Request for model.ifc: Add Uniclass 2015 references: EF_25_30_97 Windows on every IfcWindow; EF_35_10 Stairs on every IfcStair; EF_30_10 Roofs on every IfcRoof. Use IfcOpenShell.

First a look at what the model holds.

```python
import ifcopenshell

model = ifcopenshell.open("model.ifc")
print(model.schema)
print("classifications:", [c.Name for c in model.by_type("IfcClassification")])
for ifc_class in ("IfcDoor", "IfcRoof", "IfcStair", "IfcWall", "IfcWindow"):
    print(ifc_class, len(model.by_type(ifc_class)))
```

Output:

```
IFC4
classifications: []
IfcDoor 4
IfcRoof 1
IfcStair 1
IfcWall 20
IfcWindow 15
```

```python
import ifcopenshell
import ifcopenshell.api.classification

model = ifcopenshell.open("model.ifc")

system = ifcopenshell.api.classification.add_classification(model, classification="Uniclass 2015")

codes = {
    "IfcWindow": ("EF_25_30_97", "Windows"),
    "IfcStair": ("EF_35_10", "Stairs"),
    "IfcRoof": ("EF_30_10", "Roofs"),
}
for ifc_class, (code, name) in codes.items():
    products = model.by_type(ifc_class)
    ifcopenshell.api.classification.add_reference(
        model, products=products, classification=system, identification=code, name=name
    )
    print(code, len(products))

model.write("model-out.ifc")
```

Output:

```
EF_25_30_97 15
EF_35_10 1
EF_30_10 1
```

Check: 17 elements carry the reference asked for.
